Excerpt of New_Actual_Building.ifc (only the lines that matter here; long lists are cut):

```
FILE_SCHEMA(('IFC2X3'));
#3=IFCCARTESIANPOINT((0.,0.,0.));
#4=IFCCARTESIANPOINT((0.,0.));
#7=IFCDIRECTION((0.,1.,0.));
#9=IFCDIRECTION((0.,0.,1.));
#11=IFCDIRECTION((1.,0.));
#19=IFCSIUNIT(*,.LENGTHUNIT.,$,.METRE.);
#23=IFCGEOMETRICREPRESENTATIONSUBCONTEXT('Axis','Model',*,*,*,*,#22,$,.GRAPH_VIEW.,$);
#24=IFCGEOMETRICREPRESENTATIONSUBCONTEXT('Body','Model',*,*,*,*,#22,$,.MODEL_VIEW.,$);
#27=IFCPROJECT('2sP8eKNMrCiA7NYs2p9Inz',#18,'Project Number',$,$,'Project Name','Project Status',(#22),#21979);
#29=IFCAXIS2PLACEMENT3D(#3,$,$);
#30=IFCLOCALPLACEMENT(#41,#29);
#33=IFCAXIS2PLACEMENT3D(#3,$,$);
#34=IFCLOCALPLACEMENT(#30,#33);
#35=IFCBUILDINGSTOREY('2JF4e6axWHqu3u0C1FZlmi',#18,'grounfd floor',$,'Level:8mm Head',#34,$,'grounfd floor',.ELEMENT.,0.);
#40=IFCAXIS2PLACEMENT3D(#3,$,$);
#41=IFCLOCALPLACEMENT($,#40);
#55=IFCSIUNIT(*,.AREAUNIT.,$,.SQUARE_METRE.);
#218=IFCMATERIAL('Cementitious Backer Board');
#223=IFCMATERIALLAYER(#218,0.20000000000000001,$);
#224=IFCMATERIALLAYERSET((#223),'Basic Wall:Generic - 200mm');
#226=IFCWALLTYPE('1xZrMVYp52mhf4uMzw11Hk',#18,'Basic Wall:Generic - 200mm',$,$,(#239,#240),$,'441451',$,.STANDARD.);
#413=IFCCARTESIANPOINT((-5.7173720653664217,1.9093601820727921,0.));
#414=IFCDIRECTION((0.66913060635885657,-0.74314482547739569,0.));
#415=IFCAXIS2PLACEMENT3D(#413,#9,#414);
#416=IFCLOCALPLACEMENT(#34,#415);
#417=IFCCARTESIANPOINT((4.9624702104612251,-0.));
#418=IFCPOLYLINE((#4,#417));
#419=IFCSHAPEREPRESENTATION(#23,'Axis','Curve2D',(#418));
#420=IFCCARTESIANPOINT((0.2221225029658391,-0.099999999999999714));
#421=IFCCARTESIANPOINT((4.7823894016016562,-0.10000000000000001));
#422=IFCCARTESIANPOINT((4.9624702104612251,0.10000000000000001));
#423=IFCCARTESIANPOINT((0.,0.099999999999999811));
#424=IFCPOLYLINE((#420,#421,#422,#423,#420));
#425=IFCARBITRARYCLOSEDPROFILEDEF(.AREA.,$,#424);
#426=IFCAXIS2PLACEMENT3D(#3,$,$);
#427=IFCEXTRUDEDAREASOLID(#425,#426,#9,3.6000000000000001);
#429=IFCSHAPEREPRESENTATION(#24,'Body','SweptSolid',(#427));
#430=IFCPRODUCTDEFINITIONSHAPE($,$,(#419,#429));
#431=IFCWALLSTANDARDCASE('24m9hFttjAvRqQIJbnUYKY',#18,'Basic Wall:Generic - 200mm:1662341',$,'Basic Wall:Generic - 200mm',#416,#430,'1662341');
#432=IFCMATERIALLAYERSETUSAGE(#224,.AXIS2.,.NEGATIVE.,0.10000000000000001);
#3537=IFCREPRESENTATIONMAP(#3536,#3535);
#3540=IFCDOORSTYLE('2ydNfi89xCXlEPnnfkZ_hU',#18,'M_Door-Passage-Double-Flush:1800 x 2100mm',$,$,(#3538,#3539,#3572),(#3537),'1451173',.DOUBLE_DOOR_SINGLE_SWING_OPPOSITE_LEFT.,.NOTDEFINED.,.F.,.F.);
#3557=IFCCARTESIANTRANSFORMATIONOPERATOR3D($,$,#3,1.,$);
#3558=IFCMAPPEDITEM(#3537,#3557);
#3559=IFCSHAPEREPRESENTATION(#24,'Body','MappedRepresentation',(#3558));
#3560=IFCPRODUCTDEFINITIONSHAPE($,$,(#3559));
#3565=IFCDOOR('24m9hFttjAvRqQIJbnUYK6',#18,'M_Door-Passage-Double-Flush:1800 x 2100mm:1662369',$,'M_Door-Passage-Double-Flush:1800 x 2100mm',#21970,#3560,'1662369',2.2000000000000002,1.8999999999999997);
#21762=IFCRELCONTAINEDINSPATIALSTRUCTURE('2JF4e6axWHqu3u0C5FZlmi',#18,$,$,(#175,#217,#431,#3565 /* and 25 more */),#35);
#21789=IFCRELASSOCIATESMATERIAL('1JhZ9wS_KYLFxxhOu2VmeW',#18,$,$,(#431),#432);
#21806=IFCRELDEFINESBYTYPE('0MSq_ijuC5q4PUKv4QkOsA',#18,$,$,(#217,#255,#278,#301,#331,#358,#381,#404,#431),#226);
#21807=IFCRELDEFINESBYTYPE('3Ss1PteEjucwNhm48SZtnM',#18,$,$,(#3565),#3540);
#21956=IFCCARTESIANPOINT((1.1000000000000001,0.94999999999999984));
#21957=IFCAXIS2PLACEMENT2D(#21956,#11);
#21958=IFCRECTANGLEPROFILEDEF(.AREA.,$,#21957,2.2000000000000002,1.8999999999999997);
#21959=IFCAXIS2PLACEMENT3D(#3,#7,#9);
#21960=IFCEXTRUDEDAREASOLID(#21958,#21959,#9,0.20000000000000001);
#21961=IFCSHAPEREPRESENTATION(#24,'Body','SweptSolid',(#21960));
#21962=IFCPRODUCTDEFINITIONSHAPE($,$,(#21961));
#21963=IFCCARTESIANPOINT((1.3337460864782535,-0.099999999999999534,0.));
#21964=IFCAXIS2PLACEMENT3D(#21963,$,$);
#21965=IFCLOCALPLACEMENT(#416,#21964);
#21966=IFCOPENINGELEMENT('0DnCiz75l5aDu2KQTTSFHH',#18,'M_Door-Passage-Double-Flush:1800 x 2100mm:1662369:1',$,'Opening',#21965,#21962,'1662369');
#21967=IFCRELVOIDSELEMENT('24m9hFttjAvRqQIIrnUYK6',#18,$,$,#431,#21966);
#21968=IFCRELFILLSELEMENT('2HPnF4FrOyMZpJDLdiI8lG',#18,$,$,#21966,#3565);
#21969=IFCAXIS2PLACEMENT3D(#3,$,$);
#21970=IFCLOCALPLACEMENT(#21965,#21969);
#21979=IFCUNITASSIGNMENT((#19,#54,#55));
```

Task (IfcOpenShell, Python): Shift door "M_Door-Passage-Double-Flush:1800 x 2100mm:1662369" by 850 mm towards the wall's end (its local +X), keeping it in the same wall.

```python
import ifcopenshell
import ifcopenshell.api.geometry
import ifcopenshell.util.placement

model = ifcopenshell.open("New_Actual_Building.ifc")

door = model.by_guid("24m9hFttjAvRqQIJbnUYK6")
opening = door.FillsVoids[0].RelatingOpeningElement
wall = opening.VoidsElements[0].RelatingBuildingElement

wall_matrix = ifcopenshell.util.placement.get_local_placement(wall.ObjectPlacement)
shift = wall_matrix[:3, 0] * 0.85
before = ifcopenshell.util.placement.get_local_placement(door.ObjectPlacement)[:3, 3].copy()

# The door is placed relative to its opening, so it follows when the opening moves.
matrix = ifcopenshell.util.placement.get_local_placement(opening.ObjectPlacement)
matrix[:3, 3] += shift
ifcopenshell.api.geometry.edit_object_placement(
    model, product=opening, matrix=matrix, is_si=False, should_transform_children=True
)

after = ifcopenshell.util.placement.get_local_placement(door.ObjectPlacement)[:3, 3]
print("door moved by", (after - before).round(3) + 0.0)

model.write("New_Actual_Building_updated.ifc")
```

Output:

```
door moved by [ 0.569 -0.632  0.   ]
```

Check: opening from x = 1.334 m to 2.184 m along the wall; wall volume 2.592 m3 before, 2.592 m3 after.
